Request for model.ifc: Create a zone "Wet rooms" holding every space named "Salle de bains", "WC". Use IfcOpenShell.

First a look at what the model holds.

```python
import ifcopenshell

model = ifcopenshell.open("model.ifc")
print(model.schema)
seen = {}
for space in model.by_type("IfcSpace"):
    seen[space.LongName] = seen.get(space.LongName, 0) + 1
for name, count in sorted(seen.items(), key=str):
    print(count, "x", name)
print("zones:", [z.Name for z in model.by_type("IfcZone")][:20])
```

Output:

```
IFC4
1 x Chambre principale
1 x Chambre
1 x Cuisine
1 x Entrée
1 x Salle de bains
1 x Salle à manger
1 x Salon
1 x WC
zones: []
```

```python
import ifcopenshell
import ifcopenshell.api.group
import ifcopenshell.api.root

model = ifcopenshell.open("model.ifc")

names = {"Salle de bains", "WC"}
spaces = [s for s in model.by_type("IfcSpace") if s.LongName in names]

zone = ifcopenshell.api.root.create_entity(model, ifc_class="IfcZone", name="Wet rooms")
ifcopenshell.api.group.assign_group(model, products=spaces, group=zone)
print(len(spaces), "spaces in", zone.Name)

model.write("model_rev.ifc")
```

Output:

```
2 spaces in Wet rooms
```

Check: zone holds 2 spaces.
